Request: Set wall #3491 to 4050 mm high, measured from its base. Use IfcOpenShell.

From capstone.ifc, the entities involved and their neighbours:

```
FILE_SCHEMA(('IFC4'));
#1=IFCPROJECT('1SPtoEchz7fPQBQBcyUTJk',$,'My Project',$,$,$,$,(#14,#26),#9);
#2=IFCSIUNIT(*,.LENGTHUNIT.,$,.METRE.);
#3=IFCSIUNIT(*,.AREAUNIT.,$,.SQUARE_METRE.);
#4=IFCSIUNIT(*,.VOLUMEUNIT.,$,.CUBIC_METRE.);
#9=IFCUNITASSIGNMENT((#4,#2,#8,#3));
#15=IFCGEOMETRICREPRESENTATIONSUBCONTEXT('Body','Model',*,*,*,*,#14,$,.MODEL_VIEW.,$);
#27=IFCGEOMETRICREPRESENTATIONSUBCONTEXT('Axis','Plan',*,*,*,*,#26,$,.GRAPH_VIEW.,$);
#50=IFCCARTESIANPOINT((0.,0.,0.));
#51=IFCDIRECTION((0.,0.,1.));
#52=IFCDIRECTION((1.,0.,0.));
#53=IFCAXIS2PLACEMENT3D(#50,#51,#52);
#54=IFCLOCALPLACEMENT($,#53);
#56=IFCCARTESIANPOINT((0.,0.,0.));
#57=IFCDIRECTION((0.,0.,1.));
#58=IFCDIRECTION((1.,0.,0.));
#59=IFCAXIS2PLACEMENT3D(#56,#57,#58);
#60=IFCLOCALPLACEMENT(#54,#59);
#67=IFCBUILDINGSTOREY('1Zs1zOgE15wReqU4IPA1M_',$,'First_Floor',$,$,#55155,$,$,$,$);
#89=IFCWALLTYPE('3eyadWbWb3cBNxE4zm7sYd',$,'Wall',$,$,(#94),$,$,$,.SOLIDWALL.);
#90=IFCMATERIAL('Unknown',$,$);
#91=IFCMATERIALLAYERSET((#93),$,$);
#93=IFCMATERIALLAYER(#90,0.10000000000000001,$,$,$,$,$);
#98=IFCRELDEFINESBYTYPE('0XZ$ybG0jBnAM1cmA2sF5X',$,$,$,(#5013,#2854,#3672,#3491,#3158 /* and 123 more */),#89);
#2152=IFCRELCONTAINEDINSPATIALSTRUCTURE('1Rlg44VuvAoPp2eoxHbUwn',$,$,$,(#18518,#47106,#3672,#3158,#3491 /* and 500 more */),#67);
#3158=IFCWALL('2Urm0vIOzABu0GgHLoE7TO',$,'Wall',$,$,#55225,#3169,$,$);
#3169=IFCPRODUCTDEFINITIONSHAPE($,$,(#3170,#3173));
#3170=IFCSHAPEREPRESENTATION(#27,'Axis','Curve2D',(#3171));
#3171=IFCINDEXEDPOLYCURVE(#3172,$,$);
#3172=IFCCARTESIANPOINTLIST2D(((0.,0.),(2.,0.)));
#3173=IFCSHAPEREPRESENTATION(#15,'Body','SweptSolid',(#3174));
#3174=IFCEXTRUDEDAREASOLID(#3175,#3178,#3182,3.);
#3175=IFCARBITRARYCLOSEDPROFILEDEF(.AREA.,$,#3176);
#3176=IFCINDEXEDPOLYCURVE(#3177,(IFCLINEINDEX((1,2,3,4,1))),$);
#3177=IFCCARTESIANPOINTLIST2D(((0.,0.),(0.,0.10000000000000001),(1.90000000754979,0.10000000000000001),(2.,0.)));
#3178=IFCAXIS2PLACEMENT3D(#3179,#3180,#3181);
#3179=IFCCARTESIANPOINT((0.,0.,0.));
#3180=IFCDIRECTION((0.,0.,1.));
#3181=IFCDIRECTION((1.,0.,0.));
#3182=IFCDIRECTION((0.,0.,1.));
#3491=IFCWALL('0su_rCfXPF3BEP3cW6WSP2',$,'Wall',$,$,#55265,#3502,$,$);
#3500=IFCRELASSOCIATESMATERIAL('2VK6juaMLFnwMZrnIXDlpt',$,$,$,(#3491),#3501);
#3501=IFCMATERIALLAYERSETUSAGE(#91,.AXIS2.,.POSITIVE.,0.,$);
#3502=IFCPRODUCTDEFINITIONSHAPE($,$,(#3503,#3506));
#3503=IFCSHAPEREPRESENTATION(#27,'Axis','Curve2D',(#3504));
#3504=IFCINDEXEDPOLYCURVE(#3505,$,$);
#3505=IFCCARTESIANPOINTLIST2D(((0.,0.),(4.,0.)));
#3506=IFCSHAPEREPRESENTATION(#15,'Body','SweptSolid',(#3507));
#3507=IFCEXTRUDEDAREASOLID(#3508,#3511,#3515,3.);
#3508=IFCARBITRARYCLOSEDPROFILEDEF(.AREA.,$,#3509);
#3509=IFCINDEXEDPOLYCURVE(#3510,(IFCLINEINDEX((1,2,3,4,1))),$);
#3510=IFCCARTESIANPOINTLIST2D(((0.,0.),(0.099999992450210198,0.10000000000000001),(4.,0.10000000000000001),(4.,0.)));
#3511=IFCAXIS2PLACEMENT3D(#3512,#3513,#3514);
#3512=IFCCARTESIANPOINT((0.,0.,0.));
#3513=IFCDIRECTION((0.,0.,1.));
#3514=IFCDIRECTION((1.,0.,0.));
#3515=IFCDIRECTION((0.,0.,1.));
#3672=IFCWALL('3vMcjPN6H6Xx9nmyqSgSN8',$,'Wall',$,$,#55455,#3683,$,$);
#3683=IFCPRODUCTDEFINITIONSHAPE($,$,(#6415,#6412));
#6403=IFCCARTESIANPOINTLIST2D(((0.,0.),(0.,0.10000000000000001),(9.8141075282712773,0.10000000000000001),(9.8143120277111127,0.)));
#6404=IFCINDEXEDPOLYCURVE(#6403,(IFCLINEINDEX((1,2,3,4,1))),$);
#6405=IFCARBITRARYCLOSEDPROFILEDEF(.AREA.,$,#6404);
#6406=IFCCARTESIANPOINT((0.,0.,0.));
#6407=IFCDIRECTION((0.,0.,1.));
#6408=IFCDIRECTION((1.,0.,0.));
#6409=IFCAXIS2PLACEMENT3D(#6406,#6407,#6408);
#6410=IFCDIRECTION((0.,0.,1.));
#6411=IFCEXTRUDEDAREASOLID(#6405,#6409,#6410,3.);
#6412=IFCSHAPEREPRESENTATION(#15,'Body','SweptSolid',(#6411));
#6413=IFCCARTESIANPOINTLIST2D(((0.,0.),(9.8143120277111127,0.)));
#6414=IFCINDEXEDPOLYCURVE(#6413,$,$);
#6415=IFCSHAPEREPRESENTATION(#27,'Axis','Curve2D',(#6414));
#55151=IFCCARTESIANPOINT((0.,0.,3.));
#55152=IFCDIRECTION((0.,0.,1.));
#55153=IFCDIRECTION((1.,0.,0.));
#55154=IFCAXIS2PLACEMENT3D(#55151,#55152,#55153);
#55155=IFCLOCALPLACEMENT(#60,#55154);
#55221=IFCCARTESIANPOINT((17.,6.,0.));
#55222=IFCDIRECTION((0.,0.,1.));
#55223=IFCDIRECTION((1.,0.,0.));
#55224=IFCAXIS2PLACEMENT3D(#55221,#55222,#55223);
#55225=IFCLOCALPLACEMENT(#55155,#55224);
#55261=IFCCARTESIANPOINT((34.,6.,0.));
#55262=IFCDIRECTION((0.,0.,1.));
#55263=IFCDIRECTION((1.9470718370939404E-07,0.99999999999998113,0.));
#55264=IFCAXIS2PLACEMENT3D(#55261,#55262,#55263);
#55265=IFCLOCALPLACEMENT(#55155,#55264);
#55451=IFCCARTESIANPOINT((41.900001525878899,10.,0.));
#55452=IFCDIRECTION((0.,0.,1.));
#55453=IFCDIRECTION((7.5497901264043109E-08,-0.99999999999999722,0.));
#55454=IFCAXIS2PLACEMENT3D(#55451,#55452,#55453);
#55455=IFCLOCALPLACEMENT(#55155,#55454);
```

```python
import ifcopenshell
import ifcopenshell.geom
import ifcopenshell.util.representation
import ifcopenshell.util.shape
import ifcopenshell.util.unit

model = ifcopenshell.open("capstone.ifc")
unit_scale = ifcopenshell.util.unit.calculate_unit_scale(model)
settings = ifcopenshell.geom.settings()


def volume(element):
    """Net volume in cubic metres, openings subtracted."""
    shape = ifcopenshell.geom.create_shape(settings, element)
    return ifcopenshell.util.shape.get_volume(shape.geometry)


wall = model.by_id(3491)
before = volume(wall)

body = ifcopenshell.util.representation.get_representation(wall, "Model", "Body")
solid = body.Items[0]
old_height = solid.Depth
solid.Depth = 4.05 / unit_scale
after = volume(wall)

print(f"height {old_height:g} -> {solid.Depth:g}, volume {before:.3f} -> {after:.3f} m3")

model.write("capstone_rev.ifc")
```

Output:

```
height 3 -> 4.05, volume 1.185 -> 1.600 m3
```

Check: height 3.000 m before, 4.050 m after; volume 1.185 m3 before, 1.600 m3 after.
